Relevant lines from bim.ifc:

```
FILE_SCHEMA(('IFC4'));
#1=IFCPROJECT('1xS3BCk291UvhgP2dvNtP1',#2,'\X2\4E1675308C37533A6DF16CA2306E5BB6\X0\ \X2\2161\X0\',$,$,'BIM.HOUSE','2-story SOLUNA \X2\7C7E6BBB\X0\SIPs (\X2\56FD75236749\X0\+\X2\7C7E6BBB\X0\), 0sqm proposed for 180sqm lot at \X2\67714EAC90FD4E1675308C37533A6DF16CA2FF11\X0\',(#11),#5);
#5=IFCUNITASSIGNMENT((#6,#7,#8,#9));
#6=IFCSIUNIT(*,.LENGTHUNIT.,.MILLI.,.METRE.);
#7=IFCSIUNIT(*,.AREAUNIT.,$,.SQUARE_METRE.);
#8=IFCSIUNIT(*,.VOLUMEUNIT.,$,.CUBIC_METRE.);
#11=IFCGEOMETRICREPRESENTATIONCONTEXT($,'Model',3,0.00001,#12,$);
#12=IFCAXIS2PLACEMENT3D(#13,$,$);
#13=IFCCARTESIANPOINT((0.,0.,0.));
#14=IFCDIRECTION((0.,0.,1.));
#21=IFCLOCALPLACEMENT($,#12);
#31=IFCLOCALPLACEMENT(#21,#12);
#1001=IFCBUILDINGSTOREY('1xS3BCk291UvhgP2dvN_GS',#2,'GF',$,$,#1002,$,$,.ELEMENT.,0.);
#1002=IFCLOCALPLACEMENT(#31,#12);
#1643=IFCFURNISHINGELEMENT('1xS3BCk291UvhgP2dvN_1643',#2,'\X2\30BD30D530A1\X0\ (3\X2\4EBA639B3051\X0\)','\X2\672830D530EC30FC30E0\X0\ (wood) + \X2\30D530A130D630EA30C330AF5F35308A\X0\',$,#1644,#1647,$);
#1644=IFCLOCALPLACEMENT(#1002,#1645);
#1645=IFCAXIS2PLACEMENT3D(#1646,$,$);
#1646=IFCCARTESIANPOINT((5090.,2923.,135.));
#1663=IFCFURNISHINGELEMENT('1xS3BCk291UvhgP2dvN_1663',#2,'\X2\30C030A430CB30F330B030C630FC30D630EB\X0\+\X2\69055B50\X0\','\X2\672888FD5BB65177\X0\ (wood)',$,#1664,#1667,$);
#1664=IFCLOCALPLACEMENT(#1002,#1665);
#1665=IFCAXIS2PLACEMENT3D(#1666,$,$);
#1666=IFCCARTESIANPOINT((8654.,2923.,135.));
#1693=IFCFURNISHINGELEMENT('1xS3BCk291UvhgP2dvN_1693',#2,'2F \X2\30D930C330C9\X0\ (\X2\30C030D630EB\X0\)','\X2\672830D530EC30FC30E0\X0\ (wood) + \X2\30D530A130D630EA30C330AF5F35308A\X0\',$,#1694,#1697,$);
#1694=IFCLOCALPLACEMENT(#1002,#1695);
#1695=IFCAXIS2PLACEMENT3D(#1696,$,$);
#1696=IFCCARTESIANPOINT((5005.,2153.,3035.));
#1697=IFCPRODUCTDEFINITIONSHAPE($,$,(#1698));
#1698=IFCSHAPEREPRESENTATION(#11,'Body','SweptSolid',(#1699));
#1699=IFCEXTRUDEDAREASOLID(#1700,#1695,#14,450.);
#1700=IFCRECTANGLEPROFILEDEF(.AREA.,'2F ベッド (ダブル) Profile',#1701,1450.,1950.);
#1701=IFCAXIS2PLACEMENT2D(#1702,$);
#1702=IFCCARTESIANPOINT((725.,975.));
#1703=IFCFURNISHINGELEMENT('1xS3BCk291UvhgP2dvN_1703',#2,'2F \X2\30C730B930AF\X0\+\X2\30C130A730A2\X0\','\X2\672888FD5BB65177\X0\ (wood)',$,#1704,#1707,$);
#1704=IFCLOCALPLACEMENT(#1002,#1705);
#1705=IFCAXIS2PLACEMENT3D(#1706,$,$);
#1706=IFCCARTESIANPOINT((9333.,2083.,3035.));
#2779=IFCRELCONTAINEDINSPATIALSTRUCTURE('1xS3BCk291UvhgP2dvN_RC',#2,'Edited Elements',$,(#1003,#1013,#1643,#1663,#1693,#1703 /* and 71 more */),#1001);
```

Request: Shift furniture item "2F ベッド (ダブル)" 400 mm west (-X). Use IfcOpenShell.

```python
import ifcopenshell
import ifcopenshell.api.geometry
import ifcopenshell.util.placement
import ifcopenshell.util.unit

model = ifcopenshell.open("bim.ifc")
unit_scale = ifcopenshell.util.unit.calculate_unit_scale(model)

item = model.by_guid("1xS3BCk291UvhgP2dvN_1693")
matrix = ifcopenshell.util.placement.get_local_placement(item.ObjectPlacement)
matrix[0, 3] -= 0.4 / unit_scale
ifcopenshell.api.geometry.edit_object_placement(model, product=item, matrix=matrix, is_si=False)

print(ifcopenshell.util.placement.get_local_placement(item.ObjectPlacement).round(3) + 0.0)

model.write("bim_updated.ifc")
```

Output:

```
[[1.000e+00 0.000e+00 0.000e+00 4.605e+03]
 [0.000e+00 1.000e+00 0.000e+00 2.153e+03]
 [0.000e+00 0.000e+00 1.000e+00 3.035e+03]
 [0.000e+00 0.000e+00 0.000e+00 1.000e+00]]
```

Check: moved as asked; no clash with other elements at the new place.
